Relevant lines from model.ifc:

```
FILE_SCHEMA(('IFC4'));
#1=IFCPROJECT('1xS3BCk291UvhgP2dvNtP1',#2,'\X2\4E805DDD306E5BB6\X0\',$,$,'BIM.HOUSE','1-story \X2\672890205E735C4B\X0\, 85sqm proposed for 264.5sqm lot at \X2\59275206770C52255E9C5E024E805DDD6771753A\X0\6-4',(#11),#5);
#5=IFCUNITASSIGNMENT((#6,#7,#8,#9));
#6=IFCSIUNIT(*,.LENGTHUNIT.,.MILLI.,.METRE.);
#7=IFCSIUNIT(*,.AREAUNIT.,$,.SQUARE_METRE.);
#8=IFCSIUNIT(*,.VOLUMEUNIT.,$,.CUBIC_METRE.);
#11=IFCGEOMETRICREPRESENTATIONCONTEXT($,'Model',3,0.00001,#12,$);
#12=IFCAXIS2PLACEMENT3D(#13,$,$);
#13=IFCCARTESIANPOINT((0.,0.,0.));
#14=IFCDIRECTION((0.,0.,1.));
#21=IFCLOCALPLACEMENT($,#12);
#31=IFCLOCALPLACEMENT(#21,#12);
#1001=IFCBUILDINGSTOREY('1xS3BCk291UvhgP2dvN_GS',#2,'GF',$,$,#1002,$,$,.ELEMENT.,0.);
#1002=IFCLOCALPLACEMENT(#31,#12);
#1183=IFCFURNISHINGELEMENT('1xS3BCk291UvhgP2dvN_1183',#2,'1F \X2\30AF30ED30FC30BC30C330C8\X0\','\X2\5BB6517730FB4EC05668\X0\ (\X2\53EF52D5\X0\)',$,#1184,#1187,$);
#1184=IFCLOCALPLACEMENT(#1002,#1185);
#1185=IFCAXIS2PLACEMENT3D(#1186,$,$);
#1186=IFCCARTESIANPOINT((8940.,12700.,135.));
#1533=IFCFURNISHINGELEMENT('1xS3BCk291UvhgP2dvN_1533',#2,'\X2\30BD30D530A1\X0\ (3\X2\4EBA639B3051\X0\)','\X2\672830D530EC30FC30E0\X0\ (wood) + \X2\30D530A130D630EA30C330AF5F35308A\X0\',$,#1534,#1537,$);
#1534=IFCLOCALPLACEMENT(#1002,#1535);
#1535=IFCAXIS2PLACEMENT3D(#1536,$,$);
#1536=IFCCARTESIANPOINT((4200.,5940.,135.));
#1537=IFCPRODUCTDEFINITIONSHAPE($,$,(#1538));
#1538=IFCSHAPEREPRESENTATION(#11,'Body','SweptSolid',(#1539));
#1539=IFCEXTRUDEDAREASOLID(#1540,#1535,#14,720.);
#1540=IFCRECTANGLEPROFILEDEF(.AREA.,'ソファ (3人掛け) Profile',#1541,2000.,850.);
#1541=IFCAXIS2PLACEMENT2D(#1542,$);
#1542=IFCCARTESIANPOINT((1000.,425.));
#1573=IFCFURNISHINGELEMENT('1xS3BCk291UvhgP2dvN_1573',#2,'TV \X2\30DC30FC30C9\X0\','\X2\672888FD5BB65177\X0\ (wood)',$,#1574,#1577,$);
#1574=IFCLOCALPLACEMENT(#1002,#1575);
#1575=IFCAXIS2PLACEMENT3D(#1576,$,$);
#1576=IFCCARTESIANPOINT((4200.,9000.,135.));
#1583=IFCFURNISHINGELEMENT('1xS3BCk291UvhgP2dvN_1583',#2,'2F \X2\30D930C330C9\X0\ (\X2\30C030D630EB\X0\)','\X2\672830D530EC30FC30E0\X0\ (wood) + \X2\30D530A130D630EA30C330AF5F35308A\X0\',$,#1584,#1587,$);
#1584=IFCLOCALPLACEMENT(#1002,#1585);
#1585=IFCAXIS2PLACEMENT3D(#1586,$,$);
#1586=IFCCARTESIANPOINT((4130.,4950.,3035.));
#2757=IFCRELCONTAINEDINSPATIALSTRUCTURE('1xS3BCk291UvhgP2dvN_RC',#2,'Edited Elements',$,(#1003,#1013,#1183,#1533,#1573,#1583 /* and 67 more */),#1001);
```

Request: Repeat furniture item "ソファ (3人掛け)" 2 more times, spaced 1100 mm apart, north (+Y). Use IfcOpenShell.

```python
import numpy as np
import ifcopenshell
import ifcopenshell.api.geometry
import ifcopenshell.api.root
import ifcopenshell.util.element
import ifcopenshell.util.placement

model = ifcopenshell.open("model.ifc")


def reuse_history(source, copy):
    """copy_class also copies each property set's owner history, people and application; keep the originals."""
    for rel in copy.IsDefinedBy:
        if rel.is_a("IfcRelDefinesByProperties") and (history := rel.RelatingPropertyDefinition.OwnerHistory):
            rel.RelatingPropertyDefinition.OwnerHistory = source.OwnerHistory
            ifcopenshell.util.element.remove_deep2(model, history)


source = model.by_guid("1xS3BCk291UvhgP2dvN_1533")
base = ifcopenshell.util.placement.get_local_placement(source.ObjectPlacement)
step = np.array([0.0, 1.0, 0.0]) * 1100.0

for i in range(1, 3):
    copy = ifcopenshell.api.root.copy_class(model, product=source)
    copy.Representation = ifcopenshell.util.element.copy_deep(
        model, source.Representation, exclude=["IfcGeometricRepresentationContext", "IfcRepresentationMap"]
    )
    reuse_history(source, copy)
    matrix = base.copy()
    matrix[:3, 3] += i * step
    print("added at", matrix[:3, 3].round(3) + 0.0)
    ifcopenshell.api.geometry.edit_object_placement(model, product=copy, matrix=matrix, is_si=False)

model.write("model_v2.ifc")
```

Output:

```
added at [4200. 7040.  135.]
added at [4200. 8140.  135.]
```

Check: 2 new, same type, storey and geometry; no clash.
